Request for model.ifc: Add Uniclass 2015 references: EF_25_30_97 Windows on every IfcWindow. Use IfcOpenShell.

First a look at what the model holds.

```python
import ifcopenshell

model = ifcopenshell.open("model.ifc")
print(model.schema)
print("classifications:", [c.Name for c in model.by_type("IfcClassification")])
for ifc_class in ("IfcDoor", "IfcRoof", "IfcStair", "IfcWall", "IfcWindow"):
    print(ifc_class, len(model.by_type(ifc_class)))
```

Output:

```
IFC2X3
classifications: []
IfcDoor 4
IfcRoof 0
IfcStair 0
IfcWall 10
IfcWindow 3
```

```python
import ifcopenshell
import ifcopenshell.api.classification

model = ifcopenshell.open("model.ifc")

# IFC2X3 requires Source and Edition and has no link from the project to the system.
system = model.create_entity("IfcClassification", Source="NBS", Edition="2015", Name="Uniclass 2015")

codes = {
    "IfcWindow": ("EF_25_30_97", "Windows"),
}
for ifc_class, (code, name) in codes.items():
    products = model.by_type(ifc_class)
    ifcopenshell.api.classification.add_reference(
        model, products=products, classification=system, identification=code, name=name
    )
    print(code, len(products))

model.write("model_v2.ifc")
```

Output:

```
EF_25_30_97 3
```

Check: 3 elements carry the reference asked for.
